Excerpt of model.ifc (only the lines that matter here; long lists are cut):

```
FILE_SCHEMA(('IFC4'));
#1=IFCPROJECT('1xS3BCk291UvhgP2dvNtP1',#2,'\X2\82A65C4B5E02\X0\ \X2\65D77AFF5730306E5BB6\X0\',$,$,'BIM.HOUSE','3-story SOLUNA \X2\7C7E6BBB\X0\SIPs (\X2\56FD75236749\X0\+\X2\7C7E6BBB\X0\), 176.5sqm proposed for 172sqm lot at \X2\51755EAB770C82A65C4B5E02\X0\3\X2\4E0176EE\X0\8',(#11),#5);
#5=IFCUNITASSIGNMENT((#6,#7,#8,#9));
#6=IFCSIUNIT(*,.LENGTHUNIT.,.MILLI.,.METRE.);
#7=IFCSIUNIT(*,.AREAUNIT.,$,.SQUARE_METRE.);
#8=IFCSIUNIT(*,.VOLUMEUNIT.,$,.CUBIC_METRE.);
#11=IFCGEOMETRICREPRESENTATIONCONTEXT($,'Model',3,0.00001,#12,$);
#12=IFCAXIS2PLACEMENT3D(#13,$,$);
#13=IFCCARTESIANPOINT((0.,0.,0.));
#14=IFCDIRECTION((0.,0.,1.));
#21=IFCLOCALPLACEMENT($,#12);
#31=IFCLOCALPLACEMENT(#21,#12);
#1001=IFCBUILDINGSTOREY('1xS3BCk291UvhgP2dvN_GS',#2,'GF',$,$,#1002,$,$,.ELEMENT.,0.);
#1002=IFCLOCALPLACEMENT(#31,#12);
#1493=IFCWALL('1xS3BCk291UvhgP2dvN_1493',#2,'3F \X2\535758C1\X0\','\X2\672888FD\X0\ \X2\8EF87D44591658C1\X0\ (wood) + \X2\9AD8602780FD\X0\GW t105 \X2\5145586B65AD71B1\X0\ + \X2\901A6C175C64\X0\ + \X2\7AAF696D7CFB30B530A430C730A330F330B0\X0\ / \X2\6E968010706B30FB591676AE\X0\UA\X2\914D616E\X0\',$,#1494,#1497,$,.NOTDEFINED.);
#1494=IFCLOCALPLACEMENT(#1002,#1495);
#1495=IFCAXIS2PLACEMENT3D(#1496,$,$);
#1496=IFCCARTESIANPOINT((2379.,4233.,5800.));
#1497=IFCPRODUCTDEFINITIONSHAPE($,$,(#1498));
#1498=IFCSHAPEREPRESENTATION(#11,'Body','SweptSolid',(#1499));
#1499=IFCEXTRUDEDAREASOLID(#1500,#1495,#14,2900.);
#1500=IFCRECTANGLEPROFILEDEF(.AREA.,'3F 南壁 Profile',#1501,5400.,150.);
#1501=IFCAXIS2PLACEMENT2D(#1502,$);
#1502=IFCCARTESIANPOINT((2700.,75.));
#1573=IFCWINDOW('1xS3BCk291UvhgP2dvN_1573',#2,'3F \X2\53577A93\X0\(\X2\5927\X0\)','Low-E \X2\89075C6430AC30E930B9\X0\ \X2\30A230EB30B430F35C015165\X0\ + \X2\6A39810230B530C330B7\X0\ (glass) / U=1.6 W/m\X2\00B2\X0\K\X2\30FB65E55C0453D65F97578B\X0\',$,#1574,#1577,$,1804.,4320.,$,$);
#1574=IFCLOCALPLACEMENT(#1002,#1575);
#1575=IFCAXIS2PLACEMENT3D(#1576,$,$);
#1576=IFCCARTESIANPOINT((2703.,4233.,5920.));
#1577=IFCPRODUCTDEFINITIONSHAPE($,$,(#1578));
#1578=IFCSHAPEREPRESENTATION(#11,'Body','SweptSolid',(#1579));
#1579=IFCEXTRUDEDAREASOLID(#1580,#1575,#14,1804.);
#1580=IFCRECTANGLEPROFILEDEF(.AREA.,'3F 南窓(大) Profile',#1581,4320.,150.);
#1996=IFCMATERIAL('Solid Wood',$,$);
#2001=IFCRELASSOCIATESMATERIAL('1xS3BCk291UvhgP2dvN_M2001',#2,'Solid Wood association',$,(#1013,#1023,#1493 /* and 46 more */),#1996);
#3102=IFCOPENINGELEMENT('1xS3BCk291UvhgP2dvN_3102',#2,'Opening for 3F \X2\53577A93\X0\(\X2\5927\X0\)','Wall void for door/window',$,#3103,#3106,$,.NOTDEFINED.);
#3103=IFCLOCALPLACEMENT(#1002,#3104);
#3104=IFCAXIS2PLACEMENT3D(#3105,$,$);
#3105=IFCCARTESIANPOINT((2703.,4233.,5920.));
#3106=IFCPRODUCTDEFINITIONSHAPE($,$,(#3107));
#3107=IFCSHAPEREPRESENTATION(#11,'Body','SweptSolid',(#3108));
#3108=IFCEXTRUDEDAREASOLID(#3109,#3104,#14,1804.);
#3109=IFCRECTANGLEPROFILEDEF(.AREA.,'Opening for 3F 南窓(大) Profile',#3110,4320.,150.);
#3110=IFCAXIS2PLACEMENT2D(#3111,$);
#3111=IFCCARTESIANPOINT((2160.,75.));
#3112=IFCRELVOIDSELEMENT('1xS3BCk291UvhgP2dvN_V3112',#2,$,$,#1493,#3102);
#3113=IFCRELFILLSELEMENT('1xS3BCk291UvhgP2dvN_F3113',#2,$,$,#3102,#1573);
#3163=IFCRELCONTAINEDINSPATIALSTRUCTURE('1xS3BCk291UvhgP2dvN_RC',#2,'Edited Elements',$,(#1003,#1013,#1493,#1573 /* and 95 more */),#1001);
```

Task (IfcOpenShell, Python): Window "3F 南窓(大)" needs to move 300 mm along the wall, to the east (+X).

```python
import ifcopenshell
import ifcopenshell.api.geometry
import ifcopenshell.util.placement

model = ifcopenshell.open("model.ifc")

window = model.by_id(1573)
opening = window.FillsVoids[0].RelatingOpeningElement
wall = opening.VoidsElements[0].RelatingBuildingElement

wall_matrix = ifcopenshell.util.placement.get_local_placement(wall.ObjectPlacement)
shift = wall_matrix[:3, 0] * 300.0
before = ifcopenshell.util.placement.get_local_placement(window.ObjectPlacement)[:3, 3].copy()

# The window is not placed relative to its opening, so move both.
for product in (opening, window):
    matrix = ifcopenshell.util.placement.get_local_placement(product.ObjectPlacement)
    matrix[:3, 3] += shift
    ifcopenshell.api.geometry.edit_object_placement(model, product=product, matrix=matrix, is_si=False)

after = ifcopenshell.util.placement.get_local_placement(window.ObjectPlacement)[:3, 3]
print("window moved by", (after - before).round(3) + 0.0)

model.write("model_edited.ifc")
```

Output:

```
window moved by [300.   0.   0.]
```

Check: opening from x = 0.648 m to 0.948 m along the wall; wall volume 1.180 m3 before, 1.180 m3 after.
